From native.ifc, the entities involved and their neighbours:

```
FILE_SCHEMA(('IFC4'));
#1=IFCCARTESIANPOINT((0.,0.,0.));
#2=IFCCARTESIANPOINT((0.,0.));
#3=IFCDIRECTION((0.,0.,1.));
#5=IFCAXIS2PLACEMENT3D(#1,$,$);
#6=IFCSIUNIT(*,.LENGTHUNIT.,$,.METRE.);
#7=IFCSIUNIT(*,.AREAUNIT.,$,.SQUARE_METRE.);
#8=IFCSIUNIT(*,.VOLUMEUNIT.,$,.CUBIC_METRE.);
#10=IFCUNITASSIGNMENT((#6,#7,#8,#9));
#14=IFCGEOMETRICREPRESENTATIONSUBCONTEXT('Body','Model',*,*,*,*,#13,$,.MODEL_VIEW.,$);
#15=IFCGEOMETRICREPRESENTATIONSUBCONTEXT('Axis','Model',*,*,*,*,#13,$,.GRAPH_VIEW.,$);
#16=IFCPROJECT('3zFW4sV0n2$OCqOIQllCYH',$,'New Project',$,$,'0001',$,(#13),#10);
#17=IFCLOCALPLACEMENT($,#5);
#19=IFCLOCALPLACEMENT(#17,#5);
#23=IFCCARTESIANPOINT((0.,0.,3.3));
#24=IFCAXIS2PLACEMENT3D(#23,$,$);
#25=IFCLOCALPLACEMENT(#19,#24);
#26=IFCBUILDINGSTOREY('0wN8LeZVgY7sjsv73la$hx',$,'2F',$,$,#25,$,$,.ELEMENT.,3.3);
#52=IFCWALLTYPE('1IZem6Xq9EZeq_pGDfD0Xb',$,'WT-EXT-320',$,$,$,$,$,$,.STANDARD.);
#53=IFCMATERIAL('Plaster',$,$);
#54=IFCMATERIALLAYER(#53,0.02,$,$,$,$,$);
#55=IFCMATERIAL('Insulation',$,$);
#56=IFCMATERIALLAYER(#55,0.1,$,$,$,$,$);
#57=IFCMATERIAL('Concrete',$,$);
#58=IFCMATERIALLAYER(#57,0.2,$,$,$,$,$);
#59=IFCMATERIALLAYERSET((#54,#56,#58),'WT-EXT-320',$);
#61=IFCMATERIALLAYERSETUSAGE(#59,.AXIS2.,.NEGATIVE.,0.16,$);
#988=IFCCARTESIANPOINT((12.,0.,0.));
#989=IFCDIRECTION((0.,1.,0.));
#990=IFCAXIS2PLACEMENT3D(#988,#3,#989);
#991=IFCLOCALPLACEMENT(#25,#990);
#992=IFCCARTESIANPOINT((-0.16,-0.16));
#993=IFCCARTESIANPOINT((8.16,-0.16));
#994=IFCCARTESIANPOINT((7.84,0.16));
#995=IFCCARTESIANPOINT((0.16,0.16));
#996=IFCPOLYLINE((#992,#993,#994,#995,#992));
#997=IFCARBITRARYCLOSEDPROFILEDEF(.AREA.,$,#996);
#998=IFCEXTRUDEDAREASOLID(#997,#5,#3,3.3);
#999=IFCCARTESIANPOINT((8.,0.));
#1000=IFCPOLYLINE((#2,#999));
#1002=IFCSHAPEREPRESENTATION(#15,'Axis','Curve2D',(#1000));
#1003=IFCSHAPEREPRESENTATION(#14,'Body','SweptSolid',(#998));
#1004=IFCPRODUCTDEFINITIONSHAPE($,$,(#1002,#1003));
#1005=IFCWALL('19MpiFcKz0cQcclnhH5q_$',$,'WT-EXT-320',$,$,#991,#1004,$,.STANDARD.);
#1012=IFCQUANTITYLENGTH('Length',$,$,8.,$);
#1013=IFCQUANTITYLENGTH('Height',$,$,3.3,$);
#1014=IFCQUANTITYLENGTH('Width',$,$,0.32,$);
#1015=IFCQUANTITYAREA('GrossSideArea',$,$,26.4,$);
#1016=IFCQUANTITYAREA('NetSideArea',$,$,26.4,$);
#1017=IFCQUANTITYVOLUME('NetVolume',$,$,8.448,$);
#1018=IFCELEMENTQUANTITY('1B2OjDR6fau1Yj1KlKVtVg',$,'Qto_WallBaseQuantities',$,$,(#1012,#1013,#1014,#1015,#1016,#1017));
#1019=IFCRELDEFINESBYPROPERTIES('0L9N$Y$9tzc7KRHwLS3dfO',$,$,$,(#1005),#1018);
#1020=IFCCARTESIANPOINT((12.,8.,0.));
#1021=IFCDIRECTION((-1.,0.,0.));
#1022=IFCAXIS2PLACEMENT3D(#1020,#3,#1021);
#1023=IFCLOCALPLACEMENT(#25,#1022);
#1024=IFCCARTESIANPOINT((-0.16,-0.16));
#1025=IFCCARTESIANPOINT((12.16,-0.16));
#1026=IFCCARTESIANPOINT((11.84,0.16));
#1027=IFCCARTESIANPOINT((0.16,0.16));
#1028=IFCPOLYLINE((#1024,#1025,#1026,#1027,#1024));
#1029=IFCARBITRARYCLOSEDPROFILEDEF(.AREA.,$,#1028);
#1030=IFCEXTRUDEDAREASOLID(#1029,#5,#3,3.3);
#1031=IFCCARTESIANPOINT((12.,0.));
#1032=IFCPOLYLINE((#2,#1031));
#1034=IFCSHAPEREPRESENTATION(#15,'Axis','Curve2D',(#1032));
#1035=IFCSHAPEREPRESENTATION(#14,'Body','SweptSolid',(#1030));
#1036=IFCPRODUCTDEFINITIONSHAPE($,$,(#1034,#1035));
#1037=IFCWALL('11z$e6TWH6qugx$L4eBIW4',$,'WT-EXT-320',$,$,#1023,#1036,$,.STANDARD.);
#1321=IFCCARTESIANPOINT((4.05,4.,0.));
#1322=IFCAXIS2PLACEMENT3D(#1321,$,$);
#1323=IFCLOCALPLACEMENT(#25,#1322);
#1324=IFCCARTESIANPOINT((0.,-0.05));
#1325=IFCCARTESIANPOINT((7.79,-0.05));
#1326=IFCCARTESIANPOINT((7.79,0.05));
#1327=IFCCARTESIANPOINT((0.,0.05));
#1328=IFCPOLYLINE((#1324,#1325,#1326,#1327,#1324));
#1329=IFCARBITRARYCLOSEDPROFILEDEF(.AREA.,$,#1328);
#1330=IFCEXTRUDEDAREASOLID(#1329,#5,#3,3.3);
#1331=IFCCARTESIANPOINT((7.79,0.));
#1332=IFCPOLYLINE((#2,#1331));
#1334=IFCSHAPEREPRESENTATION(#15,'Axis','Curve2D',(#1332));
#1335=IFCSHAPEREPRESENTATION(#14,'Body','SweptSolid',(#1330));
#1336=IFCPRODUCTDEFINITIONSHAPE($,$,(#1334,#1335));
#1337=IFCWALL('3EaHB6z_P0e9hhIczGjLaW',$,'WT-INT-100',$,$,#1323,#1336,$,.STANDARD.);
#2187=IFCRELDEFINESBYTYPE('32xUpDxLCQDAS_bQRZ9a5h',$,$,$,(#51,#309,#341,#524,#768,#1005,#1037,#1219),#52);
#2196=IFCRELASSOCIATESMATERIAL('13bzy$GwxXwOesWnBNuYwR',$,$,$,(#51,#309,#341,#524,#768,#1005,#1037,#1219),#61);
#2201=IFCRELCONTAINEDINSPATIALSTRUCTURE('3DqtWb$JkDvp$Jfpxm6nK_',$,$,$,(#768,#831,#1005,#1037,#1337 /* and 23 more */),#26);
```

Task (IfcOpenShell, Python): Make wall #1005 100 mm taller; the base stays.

```python
import ifcopenshell
import ifcopenshell.api.pset
import ifcopenshell.geom
import ifcopenshell.util.element
import ifcopenshell.util.representation
import ifcopenshell.util.shape
import ifcopenshell.util.unit

model = ifcopenshell.open("native.ifc")
unit_scale = ifcopenshell.util.unit.calculate_unit_scale(model)
area_scale = ifcopenshell.util.unit.calculate_unit_scale(model, "AREAUNIT")
volume_scale = ifcopenshell.util.unit.calculate_unit_scale(model, "VOLUMEUNIT")
settings = ifcopenshell.geom.settings()


def volume(element):
    """Net volume in cubic metres, openings subtracted."""
    shape = ifcopenshell.geom.create_shape(settings, element)
    return ifcopenshell.util.shape.get_volume(shape.geometry)


wall = model.by_guid("19MpiFcKz0cQcclnhH5q_$")
before = volume(wall)

body = ifcopenshell.util.representation.get_representation(wall, "Model", "Body")
solid = body.Items[0]
old_height = solid.Depth
solid.Depth += 0.1 / unit_scale
after = volume(wall)
thickness = 0.32  # wall thickness in metres

# Update the stored height, areas and volumes.
qto = model.by_id(ifcopenshell.util.element.get_pset(wall, "Qto_WallBaseQuantities", should_inherit=False)["id"])
ifcopenshell.api.pset.edit_qto(model, qto=qto, properties={
    "Height": solid.Depth,
    "GrossSideArea": ifcopenshell.util.element.get_pset(wall, "Qto_WallBaseQuantities", "GrossSideArea") * solid.Depth / old_height,
    "NetSideArea": after / thickness / area_scale,
    "NetVolume": after / volume_scale,
})

print(f"height {old_height:g} -> {solid.Depth:g}, volume {before:.3f} -> {after:.3f} m3")

model.write("native-out.ifc")
```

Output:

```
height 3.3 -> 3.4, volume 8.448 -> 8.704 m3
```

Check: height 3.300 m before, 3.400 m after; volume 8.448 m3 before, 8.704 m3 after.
